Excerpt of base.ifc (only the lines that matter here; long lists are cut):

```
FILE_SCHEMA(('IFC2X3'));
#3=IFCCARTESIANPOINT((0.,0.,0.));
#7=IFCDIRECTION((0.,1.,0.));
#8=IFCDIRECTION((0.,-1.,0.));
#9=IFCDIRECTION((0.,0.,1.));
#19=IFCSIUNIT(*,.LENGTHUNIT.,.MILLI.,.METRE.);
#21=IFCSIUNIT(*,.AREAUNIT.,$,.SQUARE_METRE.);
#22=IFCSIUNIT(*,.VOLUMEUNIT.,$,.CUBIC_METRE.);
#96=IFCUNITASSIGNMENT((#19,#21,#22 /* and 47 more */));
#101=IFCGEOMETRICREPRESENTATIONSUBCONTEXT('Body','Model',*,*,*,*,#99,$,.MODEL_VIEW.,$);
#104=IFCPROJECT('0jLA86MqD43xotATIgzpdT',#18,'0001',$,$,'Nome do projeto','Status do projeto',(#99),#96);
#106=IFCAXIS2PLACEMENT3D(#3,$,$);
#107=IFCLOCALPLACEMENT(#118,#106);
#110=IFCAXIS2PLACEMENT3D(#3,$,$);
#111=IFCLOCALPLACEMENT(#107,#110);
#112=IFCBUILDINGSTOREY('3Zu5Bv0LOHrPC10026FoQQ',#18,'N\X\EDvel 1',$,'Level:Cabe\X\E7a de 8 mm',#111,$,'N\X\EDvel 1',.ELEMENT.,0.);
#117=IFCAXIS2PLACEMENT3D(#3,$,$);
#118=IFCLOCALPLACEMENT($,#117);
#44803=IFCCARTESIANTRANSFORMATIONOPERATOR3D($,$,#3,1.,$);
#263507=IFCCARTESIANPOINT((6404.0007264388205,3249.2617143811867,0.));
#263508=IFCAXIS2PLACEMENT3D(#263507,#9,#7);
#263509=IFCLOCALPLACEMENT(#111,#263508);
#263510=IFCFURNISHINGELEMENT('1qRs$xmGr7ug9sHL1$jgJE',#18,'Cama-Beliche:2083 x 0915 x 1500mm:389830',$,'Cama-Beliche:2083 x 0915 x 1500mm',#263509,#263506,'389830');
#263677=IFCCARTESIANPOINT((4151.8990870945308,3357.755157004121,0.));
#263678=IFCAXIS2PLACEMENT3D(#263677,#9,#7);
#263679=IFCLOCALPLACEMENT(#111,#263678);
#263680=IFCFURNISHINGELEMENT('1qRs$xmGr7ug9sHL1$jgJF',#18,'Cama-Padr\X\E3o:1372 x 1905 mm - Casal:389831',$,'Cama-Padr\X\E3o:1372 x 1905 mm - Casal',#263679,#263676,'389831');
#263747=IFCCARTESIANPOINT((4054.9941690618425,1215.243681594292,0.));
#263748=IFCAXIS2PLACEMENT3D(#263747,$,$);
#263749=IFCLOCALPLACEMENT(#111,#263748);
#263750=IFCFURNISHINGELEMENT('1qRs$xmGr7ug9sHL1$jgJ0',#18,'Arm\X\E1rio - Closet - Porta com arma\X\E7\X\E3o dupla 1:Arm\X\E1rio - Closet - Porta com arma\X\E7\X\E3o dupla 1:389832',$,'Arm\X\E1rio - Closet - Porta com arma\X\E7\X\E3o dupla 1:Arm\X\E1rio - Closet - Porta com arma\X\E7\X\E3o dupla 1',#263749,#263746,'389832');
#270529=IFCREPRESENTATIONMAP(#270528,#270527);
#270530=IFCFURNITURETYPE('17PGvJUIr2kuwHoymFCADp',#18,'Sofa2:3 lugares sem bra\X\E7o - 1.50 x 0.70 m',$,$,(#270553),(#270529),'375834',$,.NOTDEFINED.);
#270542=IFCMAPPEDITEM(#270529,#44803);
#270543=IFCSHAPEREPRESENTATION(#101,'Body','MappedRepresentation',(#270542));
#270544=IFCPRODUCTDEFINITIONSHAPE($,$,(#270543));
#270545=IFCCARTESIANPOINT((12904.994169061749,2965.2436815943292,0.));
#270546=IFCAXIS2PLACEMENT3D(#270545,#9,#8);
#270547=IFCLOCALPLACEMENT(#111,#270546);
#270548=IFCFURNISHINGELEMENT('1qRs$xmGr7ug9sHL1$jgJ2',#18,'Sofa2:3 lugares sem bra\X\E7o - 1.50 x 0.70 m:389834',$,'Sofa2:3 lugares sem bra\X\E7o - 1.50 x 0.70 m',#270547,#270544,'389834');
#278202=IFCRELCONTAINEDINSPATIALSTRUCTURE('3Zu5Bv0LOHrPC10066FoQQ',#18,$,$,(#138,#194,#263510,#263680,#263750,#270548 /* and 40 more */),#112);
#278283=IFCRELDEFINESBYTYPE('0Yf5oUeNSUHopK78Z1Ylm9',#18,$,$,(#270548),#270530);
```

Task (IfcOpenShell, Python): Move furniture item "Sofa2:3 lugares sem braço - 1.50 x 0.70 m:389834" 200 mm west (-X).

```python
import ifcopenshell
import ifcopenshell.api.geometry
import ifcopenshell.util.placement

model = ifcopenshell.open("base.ifc")

item = model.by_id(270548)
matrix = ifcopenshell.util.placement.get_local_placement(item.ObjectPlacement)
matrix[0, 3] -= 200.0
ifcopenshell.api.geometry.edit_object_placement(model, product=item, matrix=matrix, is_si=False)

print(ifcopenshell.util.placement.get_local_placement(item.ObjectPlacement).round(3) + 0.0)

model.write("base_updated.ifc")
```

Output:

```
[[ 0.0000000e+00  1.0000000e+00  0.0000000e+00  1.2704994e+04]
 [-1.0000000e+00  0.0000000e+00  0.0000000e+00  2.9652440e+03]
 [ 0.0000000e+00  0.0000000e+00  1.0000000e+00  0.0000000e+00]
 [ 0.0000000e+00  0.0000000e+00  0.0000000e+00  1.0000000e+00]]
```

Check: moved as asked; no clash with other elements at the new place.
